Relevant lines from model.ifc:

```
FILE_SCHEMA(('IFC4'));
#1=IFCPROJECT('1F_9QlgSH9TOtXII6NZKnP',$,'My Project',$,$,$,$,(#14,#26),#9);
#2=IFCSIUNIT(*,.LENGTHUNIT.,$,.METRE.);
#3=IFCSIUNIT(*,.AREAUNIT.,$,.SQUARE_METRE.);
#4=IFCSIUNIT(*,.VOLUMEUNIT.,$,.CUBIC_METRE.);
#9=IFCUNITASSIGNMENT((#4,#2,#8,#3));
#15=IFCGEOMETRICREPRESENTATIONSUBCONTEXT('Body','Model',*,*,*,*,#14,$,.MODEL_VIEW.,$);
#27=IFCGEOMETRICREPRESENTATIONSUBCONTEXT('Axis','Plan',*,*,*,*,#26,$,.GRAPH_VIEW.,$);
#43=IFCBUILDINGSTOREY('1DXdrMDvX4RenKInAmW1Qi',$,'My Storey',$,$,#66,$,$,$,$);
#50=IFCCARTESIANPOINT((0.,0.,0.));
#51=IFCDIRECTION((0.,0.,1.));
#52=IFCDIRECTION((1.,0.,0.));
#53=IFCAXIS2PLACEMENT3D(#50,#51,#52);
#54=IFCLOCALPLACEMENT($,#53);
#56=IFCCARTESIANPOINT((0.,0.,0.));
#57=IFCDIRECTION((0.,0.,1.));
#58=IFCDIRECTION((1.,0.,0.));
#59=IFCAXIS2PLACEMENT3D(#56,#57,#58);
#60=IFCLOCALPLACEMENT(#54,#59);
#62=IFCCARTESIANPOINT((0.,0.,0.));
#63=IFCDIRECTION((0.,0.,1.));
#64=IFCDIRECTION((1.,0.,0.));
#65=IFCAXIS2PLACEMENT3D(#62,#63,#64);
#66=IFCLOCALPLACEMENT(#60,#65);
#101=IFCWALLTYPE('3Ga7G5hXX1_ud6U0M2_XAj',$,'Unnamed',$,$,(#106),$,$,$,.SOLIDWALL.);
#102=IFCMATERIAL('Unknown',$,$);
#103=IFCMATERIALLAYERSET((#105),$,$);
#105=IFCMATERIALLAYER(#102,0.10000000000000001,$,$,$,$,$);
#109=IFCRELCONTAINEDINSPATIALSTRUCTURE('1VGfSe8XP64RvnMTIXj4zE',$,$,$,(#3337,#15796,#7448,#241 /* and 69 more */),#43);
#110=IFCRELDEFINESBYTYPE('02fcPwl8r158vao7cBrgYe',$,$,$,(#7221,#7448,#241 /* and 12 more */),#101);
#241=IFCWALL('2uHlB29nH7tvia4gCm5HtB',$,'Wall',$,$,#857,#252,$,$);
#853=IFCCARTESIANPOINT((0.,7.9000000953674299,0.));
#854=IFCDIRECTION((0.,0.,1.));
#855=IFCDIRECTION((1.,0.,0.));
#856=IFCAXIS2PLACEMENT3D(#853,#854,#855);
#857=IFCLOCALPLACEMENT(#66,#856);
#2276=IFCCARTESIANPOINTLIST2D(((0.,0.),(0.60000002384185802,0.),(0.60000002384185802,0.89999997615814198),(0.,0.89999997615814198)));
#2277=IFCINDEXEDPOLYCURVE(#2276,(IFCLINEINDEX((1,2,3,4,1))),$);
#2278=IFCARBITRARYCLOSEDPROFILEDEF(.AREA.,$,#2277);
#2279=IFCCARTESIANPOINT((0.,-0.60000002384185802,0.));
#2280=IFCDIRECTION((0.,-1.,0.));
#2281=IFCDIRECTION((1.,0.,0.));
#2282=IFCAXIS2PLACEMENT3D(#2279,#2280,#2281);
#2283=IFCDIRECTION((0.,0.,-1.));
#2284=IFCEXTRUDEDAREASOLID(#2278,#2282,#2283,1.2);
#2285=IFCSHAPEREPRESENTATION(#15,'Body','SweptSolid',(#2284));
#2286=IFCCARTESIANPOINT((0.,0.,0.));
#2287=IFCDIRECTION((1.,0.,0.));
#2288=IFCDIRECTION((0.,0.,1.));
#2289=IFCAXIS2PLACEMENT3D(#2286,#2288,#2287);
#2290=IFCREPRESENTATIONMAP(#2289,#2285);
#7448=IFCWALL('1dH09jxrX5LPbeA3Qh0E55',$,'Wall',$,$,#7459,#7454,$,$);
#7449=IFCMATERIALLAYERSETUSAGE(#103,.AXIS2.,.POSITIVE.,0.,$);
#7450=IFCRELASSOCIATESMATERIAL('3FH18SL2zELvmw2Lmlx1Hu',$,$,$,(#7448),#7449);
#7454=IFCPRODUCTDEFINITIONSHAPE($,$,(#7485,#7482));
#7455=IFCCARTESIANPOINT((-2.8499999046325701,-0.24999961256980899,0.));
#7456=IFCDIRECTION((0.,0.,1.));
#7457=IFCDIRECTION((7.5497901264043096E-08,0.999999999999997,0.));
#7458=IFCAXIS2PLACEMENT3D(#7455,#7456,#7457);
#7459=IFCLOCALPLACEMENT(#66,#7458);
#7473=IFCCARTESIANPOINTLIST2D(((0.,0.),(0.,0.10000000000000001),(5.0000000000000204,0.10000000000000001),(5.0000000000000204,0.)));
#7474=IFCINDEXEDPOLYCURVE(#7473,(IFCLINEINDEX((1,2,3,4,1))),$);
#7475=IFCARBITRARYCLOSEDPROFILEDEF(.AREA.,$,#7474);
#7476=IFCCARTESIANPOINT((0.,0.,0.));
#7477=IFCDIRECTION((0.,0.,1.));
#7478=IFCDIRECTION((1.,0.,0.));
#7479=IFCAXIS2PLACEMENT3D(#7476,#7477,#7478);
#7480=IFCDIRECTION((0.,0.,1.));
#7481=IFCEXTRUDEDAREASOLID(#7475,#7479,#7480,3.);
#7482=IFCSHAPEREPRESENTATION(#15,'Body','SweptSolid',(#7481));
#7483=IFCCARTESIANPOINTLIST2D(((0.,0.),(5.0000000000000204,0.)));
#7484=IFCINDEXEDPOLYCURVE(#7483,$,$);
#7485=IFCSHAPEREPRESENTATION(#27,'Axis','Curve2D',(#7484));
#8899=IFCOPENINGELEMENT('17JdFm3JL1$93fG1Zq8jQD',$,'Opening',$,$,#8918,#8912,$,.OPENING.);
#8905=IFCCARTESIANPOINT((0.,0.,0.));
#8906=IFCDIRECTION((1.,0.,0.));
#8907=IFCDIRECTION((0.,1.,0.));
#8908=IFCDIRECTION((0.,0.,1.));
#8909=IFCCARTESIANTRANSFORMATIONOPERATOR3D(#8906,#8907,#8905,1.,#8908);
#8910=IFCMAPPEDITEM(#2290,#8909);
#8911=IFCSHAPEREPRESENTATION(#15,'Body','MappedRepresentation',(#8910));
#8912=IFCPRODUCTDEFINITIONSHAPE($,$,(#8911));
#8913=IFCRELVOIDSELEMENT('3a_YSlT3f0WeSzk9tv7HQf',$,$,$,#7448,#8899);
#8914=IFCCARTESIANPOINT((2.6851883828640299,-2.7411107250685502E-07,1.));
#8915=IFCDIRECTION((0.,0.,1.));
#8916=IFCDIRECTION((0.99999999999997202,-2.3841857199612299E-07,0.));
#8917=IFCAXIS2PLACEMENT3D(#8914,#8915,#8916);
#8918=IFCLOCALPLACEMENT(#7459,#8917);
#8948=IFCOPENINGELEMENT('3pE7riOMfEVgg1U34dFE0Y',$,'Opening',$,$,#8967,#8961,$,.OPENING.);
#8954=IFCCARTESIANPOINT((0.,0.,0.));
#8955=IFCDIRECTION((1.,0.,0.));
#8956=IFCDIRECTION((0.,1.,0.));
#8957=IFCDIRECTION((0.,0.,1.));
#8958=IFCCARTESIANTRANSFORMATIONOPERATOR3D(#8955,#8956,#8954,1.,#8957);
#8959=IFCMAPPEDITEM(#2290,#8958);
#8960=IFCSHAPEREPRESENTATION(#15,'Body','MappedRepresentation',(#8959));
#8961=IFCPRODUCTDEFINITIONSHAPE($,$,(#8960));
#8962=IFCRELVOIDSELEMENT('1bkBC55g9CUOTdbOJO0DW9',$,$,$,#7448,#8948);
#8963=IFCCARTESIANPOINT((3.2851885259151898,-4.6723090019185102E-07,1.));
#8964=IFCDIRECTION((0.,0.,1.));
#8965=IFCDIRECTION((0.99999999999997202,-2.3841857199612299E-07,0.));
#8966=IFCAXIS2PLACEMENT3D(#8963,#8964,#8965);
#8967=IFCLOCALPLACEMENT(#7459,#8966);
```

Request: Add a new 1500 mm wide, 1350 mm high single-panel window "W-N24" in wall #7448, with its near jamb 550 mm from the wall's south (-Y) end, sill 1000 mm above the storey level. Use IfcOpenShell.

```python
import numpy as np
import ifcopenshell
import ifcopenshell.api.feature
import ifcopenshell.api.geometry
import ifcopenshell.api.root
import ifcopenshell.api.spatial
import ifcopenshell.geom
import ifcopenshell.util.element
import ifcopenshell.util.placement
import ifcopenshell.util.representation
import ifcopenshell.util.shape
import ifcopenshell.util.unit

model = ifcopenshell.open("model.ifc")
unit_scale = ifcopenshell.util.unit.calculate_unit_scale(model)
settings = ifcopenshell.geom.settings()


def volume(element):
    """Net volume in cubic metres, openings subtracted."""
    shape = ifcopenshell.geom.create_shape(settings, element)
    return ifcopenshell.util.shape.get_volume(shape.geometry)


wall = model.by_guid("1dH09jxrX5LPbeA3Qh0E55")
storey = ifcopenshell.util.element.get_container(wall, ifc_class="IfcBuildingStorey")
context = ifcopenshell.util.representation.get_context(model, "Model", "Body", "MODEL_VIEW")
before = volume(wall)

width, height, from_end, sill = 1.5, 1.35, 0.55, 1  # metres

# The wall runs along its own X axis, and the end named is its -X end.
wall_shape = ifcopenshell.geom.create_shape(settings, wall)
x, y, z = ifcopenshell.util.shape.get_vertices(wall_shape.geometry).T
start = x.min() + from_end
face, thickness = float(y.min()), float(y.max() - y.min())
wall_matrix = ifcopenshell.util.placement.get_local_placement(wall.ObjectPlacement)
level = ifcopenshell.util.placement.get_local_placement(storey.ObjectPlacement)[2, 3]


def in_wall(x, y):
    """Placement at x, y metres in the wall's axes, at sill height."""
    matrix = wall_matrix.copy()
    matrix[:, 3] = wall_matrix @ np.array([x / unit_scale, y / unit_scale, 0.0, 1.0])
    matrix[2, 3] = level + sill / unit_scale
    return matrix


# Opening: a box that overshoots both wall faces by 50 mm.
opening = ifcopenshell.api.root.create_entity(model, ifc_class="IfcOpeningElement", predefined_type="OPENING")
box = ifcopenshell.api.geometry.add_wall_representation(
    model, context=context, length=width, height=height, thickness=thickness + 0.1
)
ifcopenshell.api.geometry.assign_representation(model, product=opening, representation=box)
ifcopenshell.api.geometry.edit_object_placement(model, product=opening, matrix=in_wall(start, face - 0.05), is_si=False)
ifcopenshell.api.feature.add_feature(model, feature=opening, element=wall)

window = ifcopenshell.api.root.create_entity(model, ifc_class="IfcWindow", name="W-N24", predefined_type="WINDOW")
window.OverallWidth, window.OverallHeight = width / unit_scale, height / unit_scale
window.PartitioningType = "SINGLE_PANEL"
body = ifcopenshell.api.geometry.add_window_representation(
    model,
    context=context,
    overall_width=window.OverallWidth,
    overall_height=window.OverallHeight,
    partition_type="SINGLE_PANEL",
)
ifcopenshell.api.geometry.assign_representation(model, product=window, representation=body)
ifcopenshell.api.spatial.assign_container(model, products=[window], relating_structure=storey)
ifcopenshell.api.feature.add_filling(model, opening=opening, element=window)

# Centre the window in the wall's thickness.
ifcopenshell.api.geometry.edit_object_placement(model, product=window, matrix=in_wall(start, face), is_si=False)
window_shape = ifcopenshell.geom.create_shape(settings, window)
depth = ifcopenshell.util.shape.get_vertices(window_shape.geometry)[:, 1]
offset = face + thickness / 2 - (depth.min() + depth.max()) / 2
ifcopenshell.api.geometry.edit_object_placement(model, product=window, matrix=in_wall(start, offset), is_si=False)

after = volume(wall)

print(f"wall volume {before:.3f} -> {after:.3f} m3")

model.write("model_edited.ifc")
```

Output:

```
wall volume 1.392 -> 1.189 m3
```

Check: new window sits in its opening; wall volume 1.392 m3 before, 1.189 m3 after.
